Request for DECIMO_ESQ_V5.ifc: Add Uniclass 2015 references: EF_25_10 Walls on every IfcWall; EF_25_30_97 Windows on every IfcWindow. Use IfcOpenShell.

First a look at what the model holds.

```python
import ifcopenshell

model = ifcopenshell.open("DECIMO_ESQ_V5.ifc")
print(model.schema)
print("classifications:", [c.Name for c in model.by_type("IfcClassification")])
for ifc_class in ("IfcDoor", "IfcRoof", "IfcStair", "IfcWall", "IfcWindow"):
    print(ifc_class, len(model.by_type(ifc_class)))
```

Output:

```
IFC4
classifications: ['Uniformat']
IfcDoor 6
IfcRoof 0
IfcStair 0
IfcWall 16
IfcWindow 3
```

```python
import ifcopenshell
import ifcopenshell.api.classification

model = ifcopenshell.open("DECIMO_ESQ_V5.ifc")

system = ifcopenshell.api.classification.add_classification(model, classification="Uniclass 2015")

codes = {
    "IfcWall": ("EF_25_10", "Walls"),
    "IfcWindow": ("EF_25_30_97", "Windows"),
}
for ifc_class, (code, name) in codes.items():
    products = model.by_type(ifc_class)
    ifcopenshell.api.classification.add_reference(
        model, products=products, classification=system, identification=code, name=name
    )
    print(code, len(products))

model.write("DECIMO_ESQ_V5_edited.ifc")
```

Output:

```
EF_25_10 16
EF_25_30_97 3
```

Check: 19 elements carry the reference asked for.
